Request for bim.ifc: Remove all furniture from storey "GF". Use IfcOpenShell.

First a look at what the model holds.

```python
import ifcopenshell
import ifcopenshell.util.element

model = ifcopenshell.open("bim.ifc")
print(model.schema)
storey = next(s for s in model.by_type("IfcBuildingStorey") if s.Name == "GF")
furniture = [e for e in ifcopenshell.util.element.get_decomposition(storey) if e.is_a("IfcFurnishingElement")]
seen = {}
for e in furniture:
    element_type = ifcopenshell.util.element.get_type(e)
    name = element_type.Name if element_type not in (None, e) else None
    seen[name] = seen.get(name, 0) + 1
for name, count in sorted(seen.items(), key=str):
    print(count, "x", name)
```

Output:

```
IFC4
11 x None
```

```python
import ifcopenshell
import ifcopenshell.api.root
import ifcopenshell.util.element

model = ifcopenshell.open("bim.ifc")

storey = next(s for s in model.by_type("IfcBuildingStorey") if s.Name == "GF")
furniture = [e for e in ifcopenshell.util.element.get_decomposition(storey) if e.is_a("IfcFurnishingElement")]

for e in furniture:
    ifcopenshell.api.root.remove_product(model, product=e)
print(len(furniture), "removed")

model.write("bim_edited.ifc")
```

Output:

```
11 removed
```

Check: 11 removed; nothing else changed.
